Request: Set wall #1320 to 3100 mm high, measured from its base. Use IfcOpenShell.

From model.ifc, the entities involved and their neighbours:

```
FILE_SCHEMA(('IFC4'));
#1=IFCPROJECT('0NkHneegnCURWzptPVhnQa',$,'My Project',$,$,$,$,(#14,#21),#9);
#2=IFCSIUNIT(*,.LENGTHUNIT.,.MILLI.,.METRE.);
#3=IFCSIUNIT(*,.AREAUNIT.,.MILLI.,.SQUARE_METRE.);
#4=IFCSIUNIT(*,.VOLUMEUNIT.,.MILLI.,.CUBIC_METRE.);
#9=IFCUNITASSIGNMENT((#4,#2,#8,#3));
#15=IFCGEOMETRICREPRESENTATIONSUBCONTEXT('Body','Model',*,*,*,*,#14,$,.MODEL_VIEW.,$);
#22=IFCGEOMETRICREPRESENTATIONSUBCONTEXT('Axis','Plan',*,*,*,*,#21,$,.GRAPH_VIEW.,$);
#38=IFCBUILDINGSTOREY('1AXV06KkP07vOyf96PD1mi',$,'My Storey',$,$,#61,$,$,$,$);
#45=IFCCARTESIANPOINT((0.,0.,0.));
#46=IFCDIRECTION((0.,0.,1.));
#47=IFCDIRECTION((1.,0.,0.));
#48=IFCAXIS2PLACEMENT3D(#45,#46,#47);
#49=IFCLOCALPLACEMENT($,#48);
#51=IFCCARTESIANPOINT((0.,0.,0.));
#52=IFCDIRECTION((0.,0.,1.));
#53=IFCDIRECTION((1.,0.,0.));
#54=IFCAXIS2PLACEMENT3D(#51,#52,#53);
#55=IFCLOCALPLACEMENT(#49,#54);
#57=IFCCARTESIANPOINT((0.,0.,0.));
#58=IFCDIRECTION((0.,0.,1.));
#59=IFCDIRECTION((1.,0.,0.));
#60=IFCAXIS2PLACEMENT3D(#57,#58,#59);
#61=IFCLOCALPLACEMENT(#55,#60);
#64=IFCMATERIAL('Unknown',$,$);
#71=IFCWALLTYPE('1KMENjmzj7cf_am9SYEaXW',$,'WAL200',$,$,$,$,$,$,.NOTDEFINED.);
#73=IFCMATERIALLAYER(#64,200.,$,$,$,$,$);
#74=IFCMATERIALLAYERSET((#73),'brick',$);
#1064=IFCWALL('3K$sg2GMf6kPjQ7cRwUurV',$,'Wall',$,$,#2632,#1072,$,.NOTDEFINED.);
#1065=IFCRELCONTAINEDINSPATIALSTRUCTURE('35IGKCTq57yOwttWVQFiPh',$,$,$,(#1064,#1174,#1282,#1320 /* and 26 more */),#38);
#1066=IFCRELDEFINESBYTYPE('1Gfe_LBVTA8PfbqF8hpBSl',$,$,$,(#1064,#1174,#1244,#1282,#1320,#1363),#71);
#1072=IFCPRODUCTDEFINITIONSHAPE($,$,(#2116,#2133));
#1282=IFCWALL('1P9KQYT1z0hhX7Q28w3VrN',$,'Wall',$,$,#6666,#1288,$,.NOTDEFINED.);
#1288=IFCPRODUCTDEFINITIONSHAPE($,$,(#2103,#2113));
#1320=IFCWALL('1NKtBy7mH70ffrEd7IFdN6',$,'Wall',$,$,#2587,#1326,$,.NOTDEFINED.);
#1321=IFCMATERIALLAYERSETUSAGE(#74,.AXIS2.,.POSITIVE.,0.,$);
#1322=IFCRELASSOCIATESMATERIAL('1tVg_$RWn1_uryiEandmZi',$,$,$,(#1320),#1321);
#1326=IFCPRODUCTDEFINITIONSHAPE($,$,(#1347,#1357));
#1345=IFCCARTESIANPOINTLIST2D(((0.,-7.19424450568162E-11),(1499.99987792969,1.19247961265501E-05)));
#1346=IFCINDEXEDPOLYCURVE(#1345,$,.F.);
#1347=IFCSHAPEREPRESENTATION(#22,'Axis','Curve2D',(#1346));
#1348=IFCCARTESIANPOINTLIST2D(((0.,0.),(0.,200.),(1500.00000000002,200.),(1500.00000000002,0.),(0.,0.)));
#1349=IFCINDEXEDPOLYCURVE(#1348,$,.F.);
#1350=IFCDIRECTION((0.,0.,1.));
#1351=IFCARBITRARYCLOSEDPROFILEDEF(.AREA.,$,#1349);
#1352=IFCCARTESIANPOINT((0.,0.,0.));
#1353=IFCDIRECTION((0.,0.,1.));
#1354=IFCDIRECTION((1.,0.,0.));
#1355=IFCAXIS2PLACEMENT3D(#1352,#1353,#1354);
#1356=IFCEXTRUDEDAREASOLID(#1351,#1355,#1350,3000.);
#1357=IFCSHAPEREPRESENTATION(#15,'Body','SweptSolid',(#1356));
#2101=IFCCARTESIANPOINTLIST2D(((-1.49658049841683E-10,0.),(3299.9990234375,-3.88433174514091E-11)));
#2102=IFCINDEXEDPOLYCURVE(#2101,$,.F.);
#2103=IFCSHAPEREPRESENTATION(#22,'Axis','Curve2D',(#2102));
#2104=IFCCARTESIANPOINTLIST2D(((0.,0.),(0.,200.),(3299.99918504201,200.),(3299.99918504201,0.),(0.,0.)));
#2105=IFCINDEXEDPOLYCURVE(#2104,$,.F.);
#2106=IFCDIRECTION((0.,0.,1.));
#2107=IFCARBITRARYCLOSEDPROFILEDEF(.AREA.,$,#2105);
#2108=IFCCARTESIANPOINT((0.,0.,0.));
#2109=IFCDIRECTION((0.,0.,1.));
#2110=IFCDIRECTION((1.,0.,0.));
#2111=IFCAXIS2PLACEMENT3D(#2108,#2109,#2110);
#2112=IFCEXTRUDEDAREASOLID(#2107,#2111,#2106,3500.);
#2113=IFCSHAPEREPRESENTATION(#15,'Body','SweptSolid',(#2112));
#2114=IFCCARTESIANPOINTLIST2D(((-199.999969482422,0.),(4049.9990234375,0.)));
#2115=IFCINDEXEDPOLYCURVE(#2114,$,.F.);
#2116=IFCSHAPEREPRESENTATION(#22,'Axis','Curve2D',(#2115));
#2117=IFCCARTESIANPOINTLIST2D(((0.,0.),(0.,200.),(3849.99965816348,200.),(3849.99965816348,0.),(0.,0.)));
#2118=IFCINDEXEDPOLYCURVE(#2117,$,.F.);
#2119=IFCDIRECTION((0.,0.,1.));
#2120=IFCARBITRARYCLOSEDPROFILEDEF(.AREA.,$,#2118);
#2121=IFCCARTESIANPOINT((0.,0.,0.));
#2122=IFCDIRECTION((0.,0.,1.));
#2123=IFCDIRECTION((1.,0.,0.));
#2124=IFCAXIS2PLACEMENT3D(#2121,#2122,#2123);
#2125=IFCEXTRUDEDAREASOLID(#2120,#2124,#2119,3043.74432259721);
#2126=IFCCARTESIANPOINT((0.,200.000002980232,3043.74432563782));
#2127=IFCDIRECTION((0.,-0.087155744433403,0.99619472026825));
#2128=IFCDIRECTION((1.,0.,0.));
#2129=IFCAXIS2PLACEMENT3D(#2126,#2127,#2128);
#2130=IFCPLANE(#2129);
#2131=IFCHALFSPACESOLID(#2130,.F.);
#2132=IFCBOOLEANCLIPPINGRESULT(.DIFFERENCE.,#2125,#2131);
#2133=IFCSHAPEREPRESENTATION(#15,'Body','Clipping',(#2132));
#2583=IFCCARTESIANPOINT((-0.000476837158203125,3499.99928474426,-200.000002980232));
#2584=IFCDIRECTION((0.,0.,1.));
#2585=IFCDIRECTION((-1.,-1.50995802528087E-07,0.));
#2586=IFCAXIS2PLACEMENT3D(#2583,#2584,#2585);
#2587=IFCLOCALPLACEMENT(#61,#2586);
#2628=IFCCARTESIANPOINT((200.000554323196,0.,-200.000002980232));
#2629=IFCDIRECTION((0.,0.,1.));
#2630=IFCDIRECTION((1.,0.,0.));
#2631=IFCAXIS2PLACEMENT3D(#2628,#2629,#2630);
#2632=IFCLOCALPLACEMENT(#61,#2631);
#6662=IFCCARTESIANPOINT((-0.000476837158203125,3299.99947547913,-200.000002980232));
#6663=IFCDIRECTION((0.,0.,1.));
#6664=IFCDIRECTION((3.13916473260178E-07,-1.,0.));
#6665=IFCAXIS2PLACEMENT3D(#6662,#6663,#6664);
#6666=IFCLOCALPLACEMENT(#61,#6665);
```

```python
import ifcopenshell
import ifcopenshell.geom
import ifcopenshell.util.representation
import ifcopenshell.util.shape
import ifcopenshell.util.unit

model = ifcopenshell.open("model.ifc")
unit_scale = ifcopenshell.util.unit.calculate_unit_scale(model)
settings = ifcopenshell.geom.settings()


def volume(element):
    """Net volume in cubic metres, openings subtracted."""
    shape = ifcopenshell.geom.create_shape(settings, element)
    return ifcopenshell.util.shape.get_volume(shape.geometry)


wall = model.by_guid("1NKtBy7mH70ffrEd7IFdN6")
before = volume(wall)

body = ifcopenshell.util.representation.get_representation(wall, "Model", "Body")
solid = body.Items[0]
old_height = solid.Depth
solid.Depth = 3.1 / unit_scale
after = volume(wall)

print(f"height {old_height:g} -> {solid.Depth:g}, volume {before:.3f} -> {after:.3f} m3")

model.write("model_v2.ifc")
```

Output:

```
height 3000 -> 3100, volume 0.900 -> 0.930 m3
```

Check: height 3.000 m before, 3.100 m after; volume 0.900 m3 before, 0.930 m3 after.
